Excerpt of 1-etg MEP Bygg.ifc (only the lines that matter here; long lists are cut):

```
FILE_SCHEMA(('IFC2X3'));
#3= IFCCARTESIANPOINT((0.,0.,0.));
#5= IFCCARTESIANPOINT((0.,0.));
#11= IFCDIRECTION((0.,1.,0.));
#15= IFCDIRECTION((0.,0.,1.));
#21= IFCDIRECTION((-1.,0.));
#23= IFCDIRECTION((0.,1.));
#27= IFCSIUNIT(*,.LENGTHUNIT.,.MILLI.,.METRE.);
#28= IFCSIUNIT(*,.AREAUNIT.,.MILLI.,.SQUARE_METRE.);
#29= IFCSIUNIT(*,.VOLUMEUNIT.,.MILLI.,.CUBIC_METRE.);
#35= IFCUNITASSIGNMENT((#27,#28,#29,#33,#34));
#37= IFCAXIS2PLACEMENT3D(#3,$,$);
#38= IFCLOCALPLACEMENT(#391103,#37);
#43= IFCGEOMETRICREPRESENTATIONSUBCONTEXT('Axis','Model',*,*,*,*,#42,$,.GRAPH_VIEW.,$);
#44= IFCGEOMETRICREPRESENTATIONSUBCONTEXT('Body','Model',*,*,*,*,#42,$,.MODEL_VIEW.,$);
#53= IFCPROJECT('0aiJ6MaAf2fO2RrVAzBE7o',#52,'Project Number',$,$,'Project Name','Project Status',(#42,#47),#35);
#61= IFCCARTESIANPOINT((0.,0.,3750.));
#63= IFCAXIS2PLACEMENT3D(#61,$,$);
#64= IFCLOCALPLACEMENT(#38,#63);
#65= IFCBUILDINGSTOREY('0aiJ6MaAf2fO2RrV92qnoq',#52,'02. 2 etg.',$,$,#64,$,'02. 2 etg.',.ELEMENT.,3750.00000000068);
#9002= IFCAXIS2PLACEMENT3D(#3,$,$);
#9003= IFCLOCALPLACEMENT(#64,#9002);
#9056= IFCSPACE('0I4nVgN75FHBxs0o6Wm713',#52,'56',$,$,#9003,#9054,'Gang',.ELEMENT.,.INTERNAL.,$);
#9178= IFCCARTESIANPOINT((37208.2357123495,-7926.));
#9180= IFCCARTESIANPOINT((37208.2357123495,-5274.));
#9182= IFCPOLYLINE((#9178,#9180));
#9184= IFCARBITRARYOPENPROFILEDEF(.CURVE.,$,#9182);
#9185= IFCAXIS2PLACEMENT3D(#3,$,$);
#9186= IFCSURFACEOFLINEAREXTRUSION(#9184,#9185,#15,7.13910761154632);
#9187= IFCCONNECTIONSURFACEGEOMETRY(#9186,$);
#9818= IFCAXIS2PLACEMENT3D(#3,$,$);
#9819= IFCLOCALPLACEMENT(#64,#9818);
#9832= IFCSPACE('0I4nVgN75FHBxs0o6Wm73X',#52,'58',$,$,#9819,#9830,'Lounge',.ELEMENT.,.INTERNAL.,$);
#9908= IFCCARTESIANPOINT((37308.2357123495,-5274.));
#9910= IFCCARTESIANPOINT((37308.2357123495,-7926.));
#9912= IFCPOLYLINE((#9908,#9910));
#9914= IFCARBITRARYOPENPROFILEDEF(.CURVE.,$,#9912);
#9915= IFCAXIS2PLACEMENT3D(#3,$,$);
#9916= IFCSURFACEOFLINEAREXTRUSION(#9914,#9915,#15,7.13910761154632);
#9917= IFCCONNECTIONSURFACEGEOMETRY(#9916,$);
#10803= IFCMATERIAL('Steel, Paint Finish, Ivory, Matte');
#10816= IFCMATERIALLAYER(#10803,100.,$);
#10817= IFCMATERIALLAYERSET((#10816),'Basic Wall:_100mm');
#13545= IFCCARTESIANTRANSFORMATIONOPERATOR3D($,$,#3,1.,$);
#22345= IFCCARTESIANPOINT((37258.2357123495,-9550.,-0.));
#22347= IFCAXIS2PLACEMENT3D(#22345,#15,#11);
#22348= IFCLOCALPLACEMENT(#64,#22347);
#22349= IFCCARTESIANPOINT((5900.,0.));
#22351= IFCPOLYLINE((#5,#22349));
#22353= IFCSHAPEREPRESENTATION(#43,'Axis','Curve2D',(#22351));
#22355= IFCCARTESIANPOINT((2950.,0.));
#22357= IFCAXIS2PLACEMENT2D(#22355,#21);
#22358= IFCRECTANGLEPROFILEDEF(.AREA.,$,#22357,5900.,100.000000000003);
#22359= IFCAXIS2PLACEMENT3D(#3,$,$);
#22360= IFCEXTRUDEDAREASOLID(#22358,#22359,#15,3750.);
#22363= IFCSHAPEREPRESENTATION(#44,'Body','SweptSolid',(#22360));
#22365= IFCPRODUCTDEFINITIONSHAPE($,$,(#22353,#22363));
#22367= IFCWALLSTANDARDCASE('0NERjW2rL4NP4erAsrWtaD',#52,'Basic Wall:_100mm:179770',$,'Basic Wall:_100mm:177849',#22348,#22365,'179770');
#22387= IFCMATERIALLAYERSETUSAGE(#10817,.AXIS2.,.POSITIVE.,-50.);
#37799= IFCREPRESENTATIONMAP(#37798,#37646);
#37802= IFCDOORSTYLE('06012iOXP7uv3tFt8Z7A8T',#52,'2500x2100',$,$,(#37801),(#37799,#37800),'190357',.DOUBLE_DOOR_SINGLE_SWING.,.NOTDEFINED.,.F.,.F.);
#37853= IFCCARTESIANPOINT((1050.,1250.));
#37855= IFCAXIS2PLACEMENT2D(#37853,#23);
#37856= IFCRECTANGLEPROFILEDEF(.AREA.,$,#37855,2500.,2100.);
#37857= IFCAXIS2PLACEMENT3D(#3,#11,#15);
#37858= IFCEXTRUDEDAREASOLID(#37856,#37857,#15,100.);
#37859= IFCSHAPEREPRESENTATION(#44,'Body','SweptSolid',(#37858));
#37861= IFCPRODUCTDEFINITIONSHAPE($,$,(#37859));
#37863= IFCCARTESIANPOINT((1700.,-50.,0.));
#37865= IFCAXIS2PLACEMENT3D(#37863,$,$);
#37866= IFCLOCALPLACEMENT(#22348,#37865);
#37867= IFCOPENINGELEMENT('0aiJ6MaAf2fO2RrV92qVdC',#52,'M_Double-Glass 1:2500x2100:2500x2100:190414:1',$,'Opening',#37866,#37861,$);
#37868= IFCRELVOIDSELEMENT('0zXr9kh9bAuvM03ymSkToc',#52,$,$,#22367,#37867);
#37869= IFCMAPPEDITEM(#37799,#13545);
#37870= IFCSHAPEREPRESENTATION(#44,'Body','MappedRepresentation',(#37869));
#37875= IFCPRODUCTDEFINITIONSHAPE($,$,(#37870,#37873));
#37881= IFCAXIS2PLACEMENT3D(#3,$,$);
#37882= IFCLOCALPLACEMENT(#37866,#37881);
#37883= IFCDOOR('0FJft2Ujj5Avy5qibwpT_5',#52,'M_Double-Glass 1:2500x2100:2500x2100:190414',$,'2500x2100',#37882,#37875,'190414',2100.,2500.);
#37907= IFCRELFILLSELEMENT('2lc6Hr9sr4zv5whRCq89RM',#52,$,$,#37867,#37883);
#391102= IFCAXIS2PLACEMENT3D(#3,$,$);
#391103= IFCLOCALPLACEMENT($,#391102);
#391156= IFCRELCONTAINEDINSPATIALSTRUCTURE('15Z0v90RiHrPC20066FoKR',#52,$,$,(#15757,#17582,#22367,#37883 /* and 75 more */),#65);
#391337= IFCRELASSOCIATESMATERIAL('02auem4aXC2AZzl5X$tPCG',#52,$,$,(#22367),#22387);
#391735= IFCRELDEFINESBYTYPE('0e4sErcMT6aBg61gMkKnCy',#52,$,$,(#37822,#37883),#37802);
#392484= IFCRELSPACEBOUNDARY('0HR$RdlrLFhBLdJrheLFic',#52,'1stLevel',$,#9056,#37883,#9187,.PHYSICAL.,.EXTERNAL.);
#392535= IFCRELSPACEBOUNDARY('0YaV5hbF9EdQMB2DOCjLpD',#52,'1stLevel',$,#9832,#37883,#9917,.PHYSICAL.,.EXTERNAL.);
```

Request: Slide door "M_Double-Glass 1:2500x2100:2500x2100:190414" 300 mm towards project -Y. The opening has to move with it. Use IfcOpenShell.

```python
import numpy as np
import ifcopenshell
import ifcopenshell.api.geometry
import ifcopenshell.util.placement

model = ifcopenshell.open("1-etg MEP Bygg.ifc")

door = model.by_guid("0FJft2Ujj5Avy5qibwpT_5")
opening = door.FillsVoids[0].RelatingOpeningElement
wall = opening.VoidsElements[0].RelatingBuildingElement

wall_matrix = ifcopenshell.util.placement.get_local_placement(wall.ObjectPlacement)
shift = wall_matrix[:3, 0] * -300.0
before = ifcopenshell.util.placement.get_local_placement(door.ObjectPlacement)[:3, 3].copy()

# The door is placed relative to its opening, so it follows when the opening moves.
matrix = ifcopenshell.util.placement.get_local_placement(opening.ObjectPlacement)
matrix[:3, 3] += shift
ifcopenshell.api.geometry.edit_object_placement(
    model, product=opening, matrix=matrix, is_si=False, should_transform_children=True
)

# Space boundary surfaces are stored in each space's coordinates; move them too.
for rel in door.ProvidesBoundaries:
    if not rel.ConnectionGeometry:
        continue
    surface = rel.ConnectionGeometry.SurfaceOnRelatingElement
    space_matrix = ifcopenshell.util.placement.get_local_placement(rel.RelatingSpace.ObjectPlacement)
    point = np.array(surface.Position.Location.Coordinates) + space_matrix[:3, :3].T @ shift
    surface.Position = model.createIfcAxis2Placement3D(
        model.createIfcCartesianPoint(point.tolist()), surface.Position.Axis, surface.Position.RefDirection
    )

after = ifcopenshell.util.placement.get_local_placement(door.ObjectPlacement)[:3, 3]
print("door moved by", (after - before).round(3) + 0.0)

model.write("1-etg MEP Bygg_updated.ifc")
```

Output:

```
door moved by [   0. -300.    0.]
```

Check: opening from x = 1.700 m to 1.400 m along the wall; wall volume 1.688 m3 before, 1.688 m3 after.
